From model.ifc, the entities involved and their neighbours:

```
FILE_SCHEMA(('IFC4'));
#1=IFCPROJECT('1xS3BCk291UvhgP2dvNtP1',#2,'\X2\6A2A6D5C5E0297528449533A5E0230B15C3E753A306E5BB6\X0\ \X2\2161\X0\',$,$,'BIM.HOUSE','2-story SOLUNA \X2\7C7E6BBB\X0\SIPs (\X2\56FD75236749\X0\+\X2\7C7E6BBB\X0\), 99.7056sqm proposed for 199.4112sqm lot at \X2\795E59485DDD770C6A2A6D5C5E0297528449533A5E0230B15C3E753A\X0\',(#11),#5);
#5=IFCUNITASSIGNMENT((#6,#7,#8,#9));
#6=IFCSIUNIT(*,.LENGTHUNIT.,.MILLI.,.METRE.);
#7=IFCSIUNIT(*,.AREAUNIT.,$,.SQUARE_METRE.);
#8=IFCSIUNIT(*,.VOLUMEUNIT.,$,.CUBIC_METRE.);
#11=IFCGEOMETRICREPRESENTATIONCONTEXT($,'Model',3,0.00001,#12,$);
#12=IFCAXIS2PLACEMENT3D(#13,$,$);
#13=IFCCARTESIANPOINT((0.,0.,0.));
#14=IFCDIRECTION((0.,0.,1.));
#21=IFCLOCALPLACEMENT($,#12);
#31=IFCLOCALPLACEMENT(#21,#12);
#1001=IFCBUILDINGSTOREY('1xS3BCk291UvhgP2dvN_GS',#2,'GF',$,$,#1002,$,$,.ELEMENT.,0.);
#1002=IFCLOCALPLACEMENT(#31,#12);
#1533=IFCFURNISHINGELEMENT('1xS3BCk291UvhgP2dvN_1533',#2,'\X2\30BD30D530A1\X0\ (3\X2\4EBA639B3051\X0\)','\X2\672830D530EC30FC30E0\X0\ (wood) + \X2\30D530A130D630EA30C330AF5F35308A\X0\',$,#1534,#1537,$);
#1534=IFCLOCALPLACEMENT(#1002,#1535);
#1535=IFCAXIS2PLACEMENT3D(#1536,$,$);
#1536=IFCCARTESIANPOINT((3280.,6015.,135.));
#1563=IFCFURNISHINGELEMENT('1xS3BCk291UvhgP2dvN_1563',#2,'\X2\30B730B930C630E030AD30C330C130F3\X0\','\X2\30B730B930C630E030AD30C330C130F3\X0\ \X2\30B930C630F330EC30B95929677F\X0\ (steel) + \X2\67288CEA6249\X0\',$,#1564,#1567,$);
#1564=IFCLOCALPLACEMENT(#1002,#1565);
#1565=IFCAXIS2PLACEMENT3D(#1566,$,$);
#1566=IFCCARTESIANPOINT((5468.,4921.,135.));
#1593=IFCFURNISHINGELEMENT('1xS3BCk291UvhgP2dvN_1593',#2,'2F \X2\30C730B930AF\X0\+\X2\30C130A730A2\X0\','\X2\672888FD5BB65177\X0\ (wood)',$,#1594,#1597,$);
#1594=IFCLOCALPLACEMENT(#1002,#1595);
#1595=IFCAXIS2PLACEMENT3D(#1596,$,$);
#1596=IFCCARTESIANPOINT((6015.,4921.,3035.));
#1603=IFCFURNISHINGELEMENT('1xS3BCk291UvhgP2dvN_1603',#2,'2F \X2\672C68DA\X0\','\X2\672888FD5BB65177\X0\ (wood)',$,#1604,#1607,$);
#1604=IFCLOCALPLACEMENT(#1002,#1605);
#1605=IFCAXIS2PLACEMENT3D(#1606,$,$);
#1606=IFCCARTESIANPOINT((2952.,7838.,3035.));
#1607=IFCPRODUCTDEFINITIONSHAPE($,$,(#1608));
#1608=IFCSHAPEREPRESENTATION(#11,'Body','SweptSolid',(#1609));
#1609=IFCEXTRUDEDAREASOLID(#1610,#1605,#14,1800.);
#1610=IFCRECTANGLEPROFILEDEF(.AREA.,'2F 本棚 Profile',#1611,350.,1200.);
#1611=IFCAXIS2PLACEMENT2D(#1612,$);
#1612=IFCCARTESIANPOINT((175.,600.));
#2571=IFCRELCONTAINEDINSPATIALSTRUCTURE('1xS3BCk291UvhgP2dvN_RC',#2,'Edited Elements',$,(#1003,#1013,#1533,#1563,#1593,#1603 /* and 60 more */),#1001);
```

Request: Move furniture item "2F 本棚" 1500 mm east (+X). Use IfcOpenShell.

```python
import ifcopenshell
import ifcopenshell.api.geometry
import ifcopenshell.util.placement

model = ifcopenshell.open("model.ifc")

item = model.by_id(1603)
matrix = ifcopenshell.util.placement.get_local_placement(item.ObjectPlacement)
matrix[0, 3] += 1500.0
ifcopenshell.api.geometry.edit_object_placement(model, product=item, matrix=matrix, is_si=False)

print(ifcopenshell.util.placement.get_local_placement(item.ObjectPlacement).round(3) + 0.0)

model.write("model-out.ifc")
```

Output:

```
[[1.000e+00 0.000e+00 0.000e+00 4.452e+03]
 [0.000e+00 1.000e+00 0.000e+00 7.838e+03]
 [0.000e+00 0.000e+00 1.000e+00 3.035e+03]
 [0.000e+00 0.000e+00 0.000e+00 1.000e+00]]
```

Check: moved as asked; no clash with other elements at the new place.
